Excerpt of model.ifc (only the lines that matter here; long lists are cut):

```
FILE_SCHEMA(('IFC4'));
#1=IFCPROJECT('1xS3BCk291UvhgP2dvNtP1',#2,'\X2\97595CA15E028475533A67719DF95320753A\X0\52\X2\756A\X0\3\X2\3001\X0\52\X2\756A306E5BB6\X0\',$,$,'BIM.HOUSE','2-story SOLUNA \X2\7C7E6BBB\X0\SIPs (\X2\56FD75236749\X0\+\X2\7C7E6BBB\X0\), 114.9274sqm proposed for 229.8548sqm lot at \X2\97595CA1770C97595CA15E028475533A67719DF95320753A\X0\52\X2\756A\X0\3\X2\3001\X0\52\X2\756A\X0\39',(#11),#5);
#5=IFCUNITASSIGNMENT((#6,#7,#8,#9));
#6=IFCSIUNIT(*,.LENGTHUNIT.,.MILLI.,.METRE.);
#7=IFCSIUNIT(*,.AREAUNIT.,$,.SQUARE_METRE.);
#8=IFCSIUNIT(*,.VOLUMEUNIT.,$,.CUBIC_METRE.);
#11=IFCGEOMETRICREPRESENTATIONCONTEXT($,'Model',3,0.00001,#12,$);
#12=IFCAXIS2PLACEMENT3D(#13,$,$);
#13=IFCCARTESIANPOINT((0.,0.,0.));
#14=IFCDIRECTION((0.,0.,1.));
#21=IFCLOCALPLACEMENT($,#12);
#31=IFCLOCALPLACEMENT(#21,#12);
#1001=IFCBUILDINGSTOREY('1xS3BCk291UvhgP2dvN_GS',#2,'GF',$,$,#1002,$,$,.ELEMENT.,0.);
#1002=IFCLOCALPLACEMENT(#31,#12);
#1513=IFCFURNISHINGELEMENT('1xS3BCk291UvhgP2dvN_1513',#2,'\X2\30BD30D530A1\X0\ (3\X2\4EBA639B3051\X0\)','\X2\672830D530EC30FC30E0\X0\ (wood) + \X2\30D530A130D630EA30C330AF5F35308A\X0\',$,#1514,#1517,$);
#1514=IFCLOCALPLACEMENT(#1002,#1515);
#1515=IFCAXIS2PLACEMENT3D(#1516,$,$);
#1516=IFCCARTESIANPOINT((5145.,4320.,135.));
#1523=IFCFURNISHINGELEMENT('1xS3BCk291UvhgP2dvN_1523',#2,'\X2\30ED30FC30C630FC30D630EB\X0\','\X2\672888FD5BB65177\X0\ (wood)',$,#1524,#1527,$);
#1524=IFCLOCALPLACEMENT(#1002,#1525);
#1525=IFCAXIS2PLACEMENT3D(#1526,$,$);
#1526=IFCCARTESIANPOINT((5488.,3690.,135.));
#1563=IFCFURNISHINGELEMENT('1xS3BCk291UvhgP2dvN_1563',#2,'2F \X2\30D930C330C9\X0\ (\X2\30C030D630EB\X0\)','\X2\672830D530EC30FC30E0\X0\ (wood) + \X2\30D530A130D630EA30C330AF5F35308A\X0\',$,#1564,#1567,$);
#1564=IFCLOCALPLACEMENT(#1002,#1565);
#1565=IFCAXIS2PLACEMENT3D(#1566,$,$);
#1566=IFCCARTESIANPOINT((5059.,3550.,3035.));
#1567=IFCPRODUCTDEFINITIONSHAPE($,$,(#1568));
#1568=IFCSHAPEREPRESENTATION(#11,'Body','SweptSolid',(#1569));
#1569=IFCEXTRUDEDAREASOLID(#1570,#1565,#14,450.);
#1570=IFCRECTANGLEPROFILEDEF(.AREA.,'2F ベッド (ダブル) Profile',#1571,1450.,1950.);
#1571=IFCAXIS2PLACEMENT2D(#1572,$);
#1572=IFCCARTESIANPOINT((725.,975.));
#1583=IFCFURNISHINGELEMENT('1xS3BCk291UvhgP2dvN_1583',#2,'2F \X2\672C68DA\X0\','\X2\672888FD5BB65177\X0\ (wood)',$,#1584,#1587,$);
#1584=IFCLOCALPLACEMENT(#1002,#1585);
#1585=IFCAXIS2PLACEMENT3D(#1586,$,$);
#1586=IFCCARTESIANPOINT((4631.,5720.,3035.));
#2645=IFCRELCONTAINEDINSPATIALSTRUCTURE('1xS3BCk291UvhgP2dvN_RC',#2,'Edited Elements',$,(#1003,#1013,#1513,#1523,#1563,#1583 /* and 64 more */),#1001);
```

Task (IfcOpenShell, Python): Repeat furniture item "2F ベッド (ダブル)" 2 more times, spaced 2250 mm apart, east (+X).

```python
import numpy as np
import ifcopenshell
import ifcopenshell.api.geometry
import ifcopenshell.api.root
import ifcopenshell.util.element
import ifcopenshell.util.placement
import ifcopenshell.util.unit

model = ifcopenshell.open("model.ifc")
unit_scale = ifcopenshell.util.unit.calculate_unit_scale(model)


def reuse_history(source, copy):
    """copy_class also copies each property set's owner history, people and application; keep the originals."""
    for rel in copy.IsDefinedBy:
        if rel.is_a("IfcRelDefinesByProperties") and (history := rel.RelatingPropertyDefinition.OwnerHistory):
            rel.RelatingPropertyDefinition.OwnerHistory = source.OwnerHistory
            ifcopenshell.util.element.remove_deep2(model, history)


source = model.by_id(1563)
base = ifcopenshell.util.placement.get_local_placement(source.ObjectPlacement)
step = np.array([1.0, 0.0, 0.0]) * 2.25 / unit_scale

for i in range(1, 3):
    copy = ifcopenshell.api.root.copy_class(model, product=source)
    copy.Representation = ifcopenshell.util.element.copy_deep(
        model, source.Representation, exclude=["IfcGeometricRepresentationContext", "IfcRepresentationMap"]
    )
    reuse_history(source, copy)
    matrix = base.copy()
    matrix[:3, 3] += i * step
    print("added at", matrix[:3, 3].round(3) + 0.0)
    ifcopenshell.api.geometry.edit_object_placement(model, product=copy, matrix=matrix, is_si=False)

model.write("model_edited.ifc")
```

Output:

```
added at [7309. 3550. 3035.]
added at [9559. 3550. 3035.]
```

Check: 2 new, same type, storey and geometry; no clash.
